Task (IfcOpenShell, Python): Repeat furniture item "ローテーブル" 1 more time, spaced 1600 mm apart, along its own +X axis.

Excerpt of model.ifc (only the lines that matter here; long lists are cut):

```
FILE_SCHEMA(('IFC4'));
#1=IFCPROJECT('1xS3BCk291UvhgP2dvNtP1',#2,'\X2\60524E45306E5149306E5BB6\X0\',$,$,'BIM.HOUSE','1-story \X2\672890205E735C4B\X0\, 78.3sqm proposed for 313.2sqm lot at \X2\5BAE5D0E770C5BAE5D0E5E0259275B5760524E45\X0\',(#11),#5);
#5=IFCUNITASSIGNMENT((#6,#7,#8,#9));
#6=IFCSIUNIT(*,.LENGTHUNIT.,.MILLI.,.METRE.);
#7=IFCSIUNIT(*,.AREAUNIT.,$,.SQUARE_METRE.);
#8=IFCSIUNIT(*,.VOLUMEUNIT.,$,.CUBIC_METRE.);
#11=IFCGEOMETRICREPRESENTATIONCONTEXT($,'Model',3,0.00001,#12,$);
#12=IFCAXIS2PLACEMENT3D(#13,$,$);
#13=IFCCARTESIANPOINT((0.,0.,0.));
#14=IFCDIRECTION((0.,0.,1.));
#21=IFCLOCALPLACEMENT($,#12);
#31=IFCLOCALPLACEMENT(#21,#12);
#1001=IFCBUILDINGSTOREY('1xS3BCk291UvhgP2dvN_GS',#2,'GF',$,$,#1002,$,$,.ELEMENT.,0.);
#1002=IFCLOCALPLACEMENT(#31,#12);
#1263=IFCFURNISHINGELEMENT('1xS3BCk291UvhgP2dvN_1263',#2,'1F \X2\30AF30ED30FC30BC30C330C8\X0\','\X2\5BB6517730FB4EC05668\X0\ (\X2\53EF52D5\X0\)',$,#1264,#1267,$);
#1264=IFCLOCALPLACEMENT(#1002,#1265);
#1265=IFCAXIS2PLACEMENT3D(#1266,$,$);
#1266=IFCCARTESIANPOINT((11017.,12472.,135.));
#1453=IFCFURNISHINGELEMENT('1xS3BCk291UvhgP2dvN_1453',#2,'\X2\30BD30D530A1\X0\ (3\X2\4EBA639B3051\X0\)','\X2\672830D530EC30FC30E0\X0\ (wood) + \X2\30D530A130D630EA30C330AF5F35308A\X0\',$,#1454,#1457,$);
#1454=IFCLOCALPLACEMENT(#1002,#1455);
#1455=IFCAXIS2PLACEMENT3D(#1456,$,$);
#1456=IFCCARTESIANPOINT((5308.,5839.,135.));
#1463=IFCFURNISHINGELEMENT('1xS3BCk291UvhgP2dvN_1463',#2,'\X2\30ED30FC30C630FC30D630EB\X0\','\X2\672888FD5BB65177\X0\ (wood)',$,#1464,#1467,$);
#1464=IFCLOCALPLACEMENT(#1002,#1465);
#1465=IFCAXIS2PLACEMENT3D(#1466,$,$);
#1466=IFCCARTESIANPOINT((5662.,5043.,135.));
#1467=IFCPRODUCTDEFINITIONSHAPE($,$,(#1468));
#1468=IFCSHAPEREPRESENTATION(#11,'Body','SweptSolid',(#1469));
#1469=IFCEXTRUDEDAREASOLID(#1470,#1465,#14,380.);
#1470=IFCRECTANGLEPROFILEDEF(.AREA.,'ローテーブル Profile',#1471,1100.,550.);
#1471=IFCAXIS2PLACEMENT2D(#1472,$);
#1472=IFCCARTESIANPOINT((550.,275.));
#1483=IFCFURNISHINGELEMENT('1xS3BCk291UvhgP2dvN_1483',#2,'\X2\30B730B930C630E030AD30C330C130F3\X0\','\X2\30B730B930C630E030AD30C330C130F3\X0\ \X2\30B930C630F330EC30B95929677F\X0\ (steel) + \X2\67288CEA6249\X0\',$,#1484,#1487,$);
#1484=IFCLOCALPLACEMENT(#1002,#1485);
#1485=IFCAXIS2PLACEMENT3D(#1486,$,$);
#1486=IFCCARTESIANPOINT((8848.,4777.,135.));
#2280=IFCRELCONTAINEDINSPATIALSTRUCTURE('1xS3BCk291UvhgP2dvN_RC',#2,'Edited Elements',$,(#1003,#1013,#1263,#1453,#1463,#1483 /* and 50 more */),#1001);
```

```python
import ifcopenshell
import ifcopenshell.api.geometry
import ifcopenshell.api.root
import ifcopenshell.util.element
import ifcopenshell.util.placement
import ifcopenshell.util.unit

model = ifcopenshell.open("model.ifc")
unit_scale = ifcopenshell.util.unit.calculate_unit_scale(model)


def reuse_history(source, copy):
    """copy_class also copies each property set's owner history, people and application; keep the originals."""
    for rel in copy.IsDefinedBy:
        if rel.is_a("IfcRelDefinesByProperties") and (history := rel.RelatingPropertyDefinition.OwnerHistory):
            rel.RelatingPropertyDefinition.OwnerHistory = source.OwnerHistory
            ifcopenshell.util.element.remove_deep2(model, history)


source = model.by_id(1463)
base = ifcopenshell.util.placement.get_local_placement(source.ObjectPlacement)
step = base[:3, 0] * 1.6 / unit_scale

for i in range(1, 2):
    copy = ifcopenshell.api.root.copy_class(model, product=source)
    copy.Representation = ifcopenshell.util.element.copy_deep(
        model, source.Representation, exclude=["IfcGeometricRepresentationContext", "IfcRepresentationMap"]
    )
    reuse_history(source, copy)
    matrix = base.copy()
    matrix[:3, 3] += i * step
    print("added at", matrix[:3, 3].round(3) + 0.0)
    ifcopenshell.api.geometry.edit_object_placement(model, product=copy, matrix=matrix, is_si=False)

model.write("model_edited.ifc")
```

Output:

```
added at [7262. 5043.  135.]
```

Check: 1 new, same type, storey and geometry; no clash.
